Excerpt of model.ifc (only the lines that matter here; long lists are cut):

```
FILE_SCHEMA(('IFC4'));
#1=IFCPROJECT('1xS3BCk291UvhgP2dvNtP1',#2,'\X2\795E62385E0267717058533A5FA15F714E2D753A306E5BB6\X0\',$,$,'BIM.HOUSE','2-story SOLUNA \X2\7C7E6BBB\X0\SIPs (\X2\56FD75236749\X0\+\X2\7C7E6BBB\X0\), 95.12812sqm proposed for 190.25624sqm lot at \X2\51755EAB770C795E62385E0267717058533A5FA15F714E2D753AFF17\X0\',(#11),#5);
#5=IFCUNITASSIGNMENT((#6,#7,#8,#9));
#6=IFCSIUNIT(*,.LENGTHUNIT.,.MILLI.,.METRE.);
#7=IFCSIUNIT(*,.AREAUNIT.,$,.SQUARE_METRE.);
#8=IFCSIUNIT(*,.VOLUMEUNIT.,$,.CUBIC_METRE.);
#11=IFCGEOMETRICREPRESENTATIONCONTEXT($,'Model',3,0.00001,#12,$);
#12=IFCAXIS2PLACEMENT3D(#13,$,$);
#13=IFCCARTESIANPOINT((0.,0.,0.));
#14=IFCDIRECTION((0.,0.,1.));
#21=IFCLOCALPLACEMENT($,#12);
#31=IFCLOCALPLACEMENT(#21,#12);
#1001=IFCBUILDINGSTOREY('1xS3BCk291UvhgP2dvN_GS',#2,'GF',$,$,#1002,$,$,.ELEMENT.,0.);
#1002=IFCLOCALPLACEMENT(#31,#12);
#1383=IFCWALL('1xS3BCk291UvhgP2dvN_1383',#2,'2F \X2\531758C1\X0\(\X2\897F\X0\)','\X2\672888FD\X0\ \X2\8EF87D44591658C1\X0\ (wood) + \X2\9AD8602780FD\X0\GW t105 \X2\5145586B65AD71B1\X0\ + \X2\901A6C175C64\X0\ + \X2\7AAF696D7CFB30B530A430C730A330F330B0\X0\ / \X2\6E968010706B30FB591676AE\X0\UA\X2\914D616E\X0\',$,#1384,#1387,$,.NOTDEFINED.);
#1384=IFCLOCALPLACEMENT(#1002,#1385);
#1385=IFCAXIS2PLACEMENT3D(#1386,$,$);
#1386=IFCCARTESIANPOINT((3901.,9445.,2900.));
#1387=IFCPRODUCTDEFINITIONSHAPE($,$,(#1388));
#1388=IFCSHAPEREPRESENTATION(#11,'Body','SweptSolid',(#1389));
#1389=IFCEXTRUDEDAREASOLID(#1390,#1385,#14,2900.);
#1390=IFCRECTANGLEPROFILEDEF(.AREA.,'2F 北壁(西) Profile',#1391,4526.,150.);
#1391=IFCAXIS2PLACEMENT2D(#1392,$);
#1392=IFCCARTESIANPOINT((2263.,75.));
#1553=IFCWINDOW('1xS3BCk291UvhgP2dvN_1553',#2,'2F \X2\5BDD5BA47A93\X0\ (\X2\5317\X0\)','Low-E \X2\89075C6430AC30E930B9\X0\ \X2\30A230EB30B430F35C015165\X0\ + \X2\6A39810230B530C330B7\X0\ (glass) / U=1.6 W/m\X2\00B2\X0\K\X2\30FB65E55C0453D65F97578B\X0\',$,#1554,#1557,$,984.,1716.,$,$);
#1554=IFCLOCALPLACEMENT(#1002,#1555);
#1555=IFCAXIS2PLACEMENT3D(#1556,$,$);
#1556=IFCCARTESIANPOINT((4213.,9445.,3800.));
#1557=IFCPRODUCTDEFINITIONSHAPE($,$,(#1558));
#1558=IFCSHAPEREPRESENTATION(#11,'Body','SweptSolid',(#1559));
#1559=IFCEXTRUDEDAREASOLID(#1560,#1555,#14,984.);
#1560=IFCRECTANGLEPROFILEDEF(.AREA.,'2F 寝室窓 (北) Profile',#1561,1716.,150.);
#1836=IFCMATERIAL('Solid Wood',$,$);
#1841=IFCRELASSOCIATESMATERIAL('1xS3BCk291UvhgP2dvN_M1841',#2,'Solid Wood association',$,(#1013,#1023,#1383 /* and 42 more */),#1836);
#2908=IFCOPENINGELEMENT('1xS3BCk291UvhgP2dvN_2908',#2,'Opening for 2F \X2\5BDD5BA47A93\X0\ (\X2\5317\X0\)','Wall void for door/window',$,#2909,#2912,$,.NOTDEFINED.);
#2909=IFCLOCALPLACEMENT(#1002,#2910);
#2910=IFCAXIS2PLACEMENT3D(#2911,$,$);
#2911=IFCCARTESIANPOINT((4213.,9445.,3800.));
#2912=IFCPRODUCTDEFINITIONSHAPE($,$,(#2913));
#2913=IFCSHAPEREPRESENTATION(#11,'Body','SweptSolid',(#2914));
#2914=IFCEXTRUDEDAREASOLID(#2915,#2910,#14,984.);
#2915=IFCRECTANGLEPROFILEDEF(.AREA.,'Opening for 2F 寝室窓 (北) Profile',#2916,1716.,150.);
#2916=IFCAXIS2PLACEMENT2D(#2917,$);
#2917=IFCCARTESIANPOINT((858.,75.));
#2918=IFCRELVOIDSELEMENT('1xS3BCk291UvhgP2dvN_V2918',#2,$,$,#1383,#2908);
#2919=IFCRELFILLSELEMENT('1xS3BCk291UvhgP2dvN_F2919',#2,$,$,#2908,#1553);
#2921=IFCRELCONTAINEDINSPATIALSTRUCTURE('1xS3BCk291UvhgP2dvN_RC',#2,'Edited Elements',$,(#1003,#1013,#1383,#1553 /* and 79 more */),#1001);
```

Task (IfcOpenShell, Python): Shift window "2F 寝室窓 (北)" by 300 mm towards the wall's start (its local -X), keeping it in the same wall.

```python
import ifcopenshell
import ifcopenshell.api.geometry
import ifcopenshell.util.placement

model = ifcopenshell.open("model.ifc")

window = model.by_id(1553)
opening = window.FillsVoids[0].RelatingOpeningElement
wall = opening.VoidsElements[0].RelatingBuildingElement

wall_matrix = ifcopenshell.util.placement.get_local_placement(wall.ObjectPlacement)
shift = wall_matrix[:3, 0] * -300.0
before = ifcopenshell.util.placement.get_local_placement(window.ObjectPlacement)[:3, 3].copy()

# The window is not placed relative to its opening, so move both.
for product in (opening, window):
    matrix = ifcopenshell.util.placement.get_local_placement(product.ObjectPlacement)
    matrix[:3, 3] += shift
    ifcopenshell.api.geometry.edit_object_placement(model, product=product, matrix=matrix, is_si=False)

after = ifcopenshell.util.placement.get_local_placement(window.ObjectPlacement)[:3, 3]
print("window moved by", (after - before).round(3) + 0.0)

model.write("model_rev.ifc")
```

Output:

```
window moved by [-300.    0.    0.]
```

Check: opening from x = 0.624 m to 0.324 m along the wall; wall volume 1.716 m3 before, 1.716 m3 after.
